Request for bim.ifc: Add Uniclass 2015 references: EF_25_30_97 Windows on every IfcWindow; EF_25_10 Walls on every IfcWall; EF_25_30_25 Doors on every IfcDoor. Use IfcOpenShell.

First a look at what the model holds.

```python
import ifcopenshell

model = ifcopenshell.open("bim.ifc")
print(model.schema)
print("classifications:", [c.Name for c in model.by_type("IfcClassification")])
for ifc_class in ("IfcDoor", "IfcRoof", "IfcStair", "IfcWall", "IfcWindow"):
    print(ifc_class, len(model.by_type(ifc_class)))
```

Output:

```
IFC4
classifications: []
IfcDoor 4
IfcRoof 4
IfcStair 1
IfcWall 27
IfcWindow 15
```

```python
import ifcopenshell
import ifcopenshell.api.classification

model = ifcopenshell.open("bim.ifc")

system = ifcopenshell.api.classification.add_classification(model, classification="Uniclass 2015")

codes = {
    "IfcWindow": ("EF_25_30_97", "Windows"),
    "IfcWall": ("EF_25_10", "Walls"),
    "IfcDoor": ("EF_25_30_25", "Doors"),
}
for ifc_class, (code, name) in codes.items():
    products = model.by_type(ifc_class)
    ifcopenshell.api.classification.add_reference(
        model, products=products, classification=system, identification=code, name=name
    )
    print(code, len(products))

model.write("bim_updated.ifc")
```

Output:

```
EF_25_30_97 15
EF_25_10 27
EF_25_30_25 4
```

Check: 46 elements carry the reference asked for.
